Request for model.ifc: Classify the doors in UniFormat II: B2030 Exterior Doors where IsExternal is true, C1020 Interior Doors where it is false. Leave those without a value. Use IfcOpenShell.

First a look at what the model holds.

```python
import ifcopenshell
import ifcopenshell.util.element

model = ifcopenshell.open("model.ifc")
print(model.schema)
print("classifications:", [c.Name for c in model.by_type("IfcClassification")])
values = [ifcopenshell.util.element.get_pset(e, "Pset_DoorCommon", "IsExternal") for e in model.by_type("IfcDoor")]
for value in (True, False, None):
    print("IsExternal", value, values.count(value))
```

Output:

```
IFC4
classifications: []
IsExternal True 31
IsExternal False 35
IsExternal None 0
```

```python
import ifcopenshell
import ifcopenshell.api.classification
import ifcopenshell.util.element

model = ifcopenshell.open("model.ifc")

system = ifcopenshell.api.classification.add_classification(model, classification="UniFormat II")

doors = model.by_type("IfcDoor")
external = {e: ifcopenshell.util.element.get_pset(e, "Pset_DoorCommon", "IsExternal") for e in doors}
for flag, code, name in ((True, "B2030", "Exterior Doors"), (False, "C1020", "Interior Doors")):
    products = [e for e in doors if external[e] is flag]
    ifcopenshell.api.classification.add_reference(
        model, products=products, classification=system, identification=code, name=name
    )
    print(code, len(products))

model.write("model_rev.ifc")
```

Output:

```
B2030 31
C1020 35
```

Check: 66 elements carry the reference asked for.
